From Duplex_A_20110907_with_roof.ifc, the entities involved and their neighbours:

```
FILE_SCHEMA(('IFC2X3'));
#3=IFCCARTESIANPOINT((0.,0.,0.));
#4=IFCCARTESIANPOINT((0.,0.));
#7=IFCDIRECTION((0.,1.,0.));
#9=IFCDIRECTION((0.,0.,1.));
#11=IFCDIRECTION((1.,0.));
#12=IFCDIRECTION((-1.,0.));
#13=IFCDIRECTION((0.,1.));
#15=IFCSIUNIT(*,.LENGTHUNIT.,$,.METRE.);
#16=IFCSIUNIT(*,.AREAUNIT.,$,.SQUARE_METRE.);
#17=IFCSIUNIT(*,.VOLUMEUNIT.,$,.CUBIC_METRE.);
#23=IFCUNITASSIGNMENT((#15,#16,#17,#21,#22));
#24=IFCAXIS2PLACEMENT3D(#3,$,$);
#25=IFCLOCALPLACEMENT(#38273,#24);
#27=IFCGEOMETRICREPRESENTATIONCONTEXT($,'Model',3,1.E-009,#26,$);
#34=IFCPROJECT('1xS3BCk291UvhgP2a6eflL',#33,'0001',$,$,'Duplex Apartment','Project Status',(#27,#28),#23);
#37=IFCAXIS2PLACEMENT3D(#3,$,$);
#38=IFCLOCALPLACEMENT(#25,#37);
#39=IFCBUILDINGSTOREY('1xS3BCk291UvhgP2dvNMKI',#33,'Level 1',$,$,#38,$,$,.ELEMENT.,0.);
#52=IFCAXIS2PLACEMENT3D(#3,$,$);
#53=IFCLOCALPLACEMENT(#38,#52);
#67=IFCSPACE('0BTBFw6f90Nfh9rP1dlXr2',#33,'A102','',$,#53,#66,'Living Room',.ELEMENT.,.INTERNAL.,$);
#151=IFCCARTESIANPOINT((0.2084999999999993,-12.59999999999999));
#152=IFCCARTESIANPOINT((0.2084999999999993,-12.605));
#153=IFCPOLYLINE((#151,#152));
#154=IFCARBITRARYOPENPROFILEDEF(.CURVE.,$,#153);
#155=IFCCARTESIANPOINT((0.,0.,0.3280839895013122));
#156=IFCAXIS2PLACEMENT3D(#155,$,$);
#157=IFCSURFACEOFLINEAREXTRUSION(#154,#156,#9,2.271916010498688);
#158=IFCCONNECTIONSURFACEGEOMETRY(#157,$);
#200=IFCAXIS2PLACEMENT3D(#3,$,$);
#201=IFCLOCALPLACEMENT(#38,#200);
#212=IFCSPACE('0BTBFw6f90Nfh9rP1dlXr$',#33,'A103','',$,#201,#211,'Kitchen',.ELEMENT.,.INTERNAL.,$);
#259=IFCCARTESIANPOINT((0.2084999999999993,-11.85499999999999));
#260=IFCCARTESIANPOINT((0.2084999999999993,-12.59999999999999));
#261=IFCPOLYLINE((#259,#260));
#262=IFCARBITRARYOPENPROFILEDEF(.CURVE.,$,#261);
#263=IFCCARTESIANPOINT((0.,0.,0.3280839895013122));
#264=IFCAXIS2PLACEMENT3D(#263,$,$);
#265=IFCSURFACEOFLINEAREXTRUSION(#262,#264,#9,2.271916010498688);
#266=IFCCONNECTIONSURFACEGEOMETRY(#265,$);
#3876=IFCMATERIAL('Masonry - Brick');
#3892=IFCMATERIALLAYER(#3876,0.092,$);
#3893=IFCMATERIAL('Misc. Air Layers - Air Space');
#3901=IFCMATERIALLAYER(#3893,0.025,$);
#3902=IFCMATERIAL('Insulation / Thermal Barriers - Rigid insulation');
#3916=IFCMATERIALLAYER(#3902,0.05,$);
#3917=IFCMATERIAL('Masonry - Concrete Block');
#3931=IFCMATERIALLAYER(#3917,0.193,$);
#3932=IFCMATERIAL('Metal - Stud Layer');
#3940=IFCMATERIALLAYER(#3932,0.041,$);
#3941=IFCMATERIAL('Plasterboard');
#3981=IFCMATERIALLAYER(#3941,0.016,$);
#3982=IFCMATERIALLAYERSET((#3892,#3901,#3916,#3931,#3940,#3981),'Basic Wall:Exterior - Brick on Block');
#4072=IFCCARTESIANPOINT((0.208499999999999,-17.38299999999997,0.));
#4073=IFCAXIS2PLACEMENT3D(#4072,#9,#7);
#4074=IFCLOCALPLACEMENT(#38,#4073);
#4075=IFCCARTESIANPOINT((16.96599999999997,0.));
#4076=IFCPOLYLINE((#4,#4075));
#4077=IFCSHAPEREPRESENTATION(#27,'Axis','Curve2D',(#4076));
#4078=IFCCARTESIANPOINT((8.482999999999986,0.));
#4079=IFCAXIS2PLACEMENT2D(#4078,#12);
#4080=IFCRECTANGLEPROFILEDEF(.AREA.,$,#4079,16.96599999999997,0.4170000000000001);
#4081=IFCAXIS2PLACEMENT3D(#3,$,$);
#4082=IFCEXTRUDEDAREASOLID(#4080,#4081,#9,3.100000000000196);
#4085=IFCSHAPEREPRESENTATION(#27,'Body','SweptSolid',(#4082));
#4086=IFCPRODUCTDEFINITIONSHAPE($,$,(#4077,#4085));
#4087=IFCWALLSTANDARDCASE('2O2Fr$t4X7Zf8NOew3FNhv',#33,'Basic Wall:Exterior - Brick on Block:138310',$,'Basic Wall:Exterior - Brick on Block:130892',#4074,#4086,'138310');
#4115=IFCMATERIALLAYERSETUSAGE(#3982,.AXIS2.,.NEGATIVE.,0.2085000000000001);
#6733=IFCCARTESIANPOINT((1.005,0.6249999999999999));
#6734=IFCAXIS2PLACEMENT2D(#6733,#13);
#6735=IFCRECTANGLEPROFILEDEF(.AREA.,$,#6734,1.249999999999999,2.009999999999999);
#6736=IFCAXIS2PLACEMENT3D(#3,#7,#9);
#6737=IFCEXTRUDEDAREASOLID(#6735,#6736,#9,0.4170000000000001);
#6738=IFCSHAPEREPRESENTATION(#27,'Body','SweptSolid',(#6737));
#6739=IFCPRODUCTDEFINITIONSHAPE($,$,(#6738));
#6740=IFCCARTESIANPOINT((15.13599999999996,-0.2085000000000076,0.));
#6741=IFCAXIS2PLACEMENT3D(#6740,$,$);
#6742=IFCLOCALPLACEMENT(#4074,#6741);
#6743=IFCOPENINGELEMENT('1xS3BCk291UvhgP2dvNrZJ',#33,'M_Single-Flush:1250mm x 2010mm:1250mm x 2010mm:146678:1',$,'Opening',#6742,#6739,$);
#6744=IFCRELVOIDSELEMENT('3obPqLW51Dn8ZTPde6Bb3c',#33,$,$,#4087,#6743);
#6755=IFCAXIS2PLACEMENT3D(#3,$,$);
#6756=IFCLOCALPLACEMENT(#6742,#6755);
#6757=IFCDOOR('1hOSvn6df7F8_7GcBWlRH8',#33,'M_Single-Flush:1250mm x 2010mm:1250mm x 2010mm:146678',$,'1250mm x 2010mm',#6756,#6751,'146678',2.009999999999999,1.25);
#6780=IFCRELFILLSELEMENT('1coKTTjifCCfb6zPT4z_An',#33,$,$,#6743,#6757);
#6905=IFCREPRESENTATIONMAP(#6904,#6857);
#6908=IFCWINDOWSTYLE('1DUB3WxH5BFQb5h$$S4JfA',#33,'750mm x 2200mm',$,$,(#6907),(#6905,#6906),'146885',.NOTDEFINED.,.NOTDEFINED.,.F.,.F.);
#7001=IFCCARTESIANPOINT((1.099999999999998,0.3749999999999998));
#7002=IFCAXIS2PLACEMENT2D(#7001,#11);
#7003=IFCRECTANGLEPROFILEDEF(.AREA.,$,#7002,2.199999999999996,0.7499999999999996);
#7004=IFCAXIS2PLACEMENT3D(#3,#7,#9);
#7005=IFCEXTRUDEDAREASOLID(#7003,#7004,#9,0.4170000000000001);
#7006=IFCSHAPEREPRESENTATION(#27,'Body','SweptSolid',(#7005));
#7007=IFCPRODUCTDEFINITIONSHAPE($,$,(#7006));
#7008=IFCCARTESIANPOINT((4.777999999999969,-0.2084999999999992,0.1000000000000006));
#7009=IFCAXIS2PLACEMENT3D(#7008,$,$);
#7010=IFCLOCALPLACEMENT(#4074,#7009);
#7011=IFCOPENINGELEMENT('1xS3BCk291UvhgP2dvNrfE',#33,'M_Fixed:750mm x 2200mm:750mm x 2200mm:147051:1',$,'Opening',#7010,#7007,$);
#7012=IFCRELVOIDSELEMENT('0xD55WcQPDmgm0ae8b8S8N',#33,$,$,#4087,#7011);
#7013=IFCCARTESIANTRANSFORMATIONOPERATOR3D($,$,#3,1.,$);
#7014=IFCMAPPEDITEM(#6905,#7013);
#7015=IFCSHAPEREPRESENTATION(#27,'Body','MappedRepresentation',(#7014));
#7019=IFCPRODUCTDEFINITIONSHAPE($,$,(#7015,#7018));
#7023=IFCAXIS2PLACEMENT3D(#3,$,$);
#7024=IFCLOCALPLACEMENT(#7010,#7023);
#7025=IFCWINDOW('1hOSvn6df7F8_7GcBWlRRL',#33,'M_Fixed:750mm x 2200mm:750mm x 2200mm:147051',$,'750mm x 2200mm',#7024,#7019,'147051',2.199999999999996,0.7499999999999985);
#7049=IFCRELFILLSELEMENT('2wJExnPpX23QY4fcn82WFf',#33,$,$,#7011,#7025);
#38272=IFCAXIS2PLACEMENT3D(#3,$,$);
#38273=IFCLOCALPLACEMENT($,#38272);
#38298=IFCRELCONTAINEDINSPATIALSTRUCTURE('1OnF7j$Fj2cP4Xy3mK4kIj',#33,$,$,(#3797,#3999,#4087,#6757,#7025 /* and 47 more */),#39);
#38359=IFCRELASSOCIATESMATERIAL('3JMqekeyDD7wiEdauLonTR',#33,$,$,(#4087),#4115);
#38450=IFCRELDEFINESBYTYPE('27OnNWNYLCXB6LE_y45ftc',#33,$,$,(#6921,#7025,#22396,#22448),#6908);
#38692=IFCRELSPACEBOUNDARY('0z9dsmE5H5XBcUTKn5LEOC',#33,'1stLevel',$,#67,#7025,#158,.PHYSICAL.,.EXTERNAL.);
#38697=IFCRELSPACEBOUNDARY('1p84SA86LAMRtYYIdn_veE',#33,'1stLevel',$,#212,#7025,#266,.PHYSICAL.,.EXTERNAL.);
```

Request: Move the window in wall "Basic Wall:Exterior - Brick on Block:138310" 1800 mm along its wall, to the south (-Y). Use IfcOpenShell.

```python
import numpy as np
import ifcopenshell
import ifcopenshell.api.geometry
import ifcopenshell.util.placement
import ifcopenshell.util.unit

model = ifcopenshell.open("Duplex_A_20110907_with_roof.ifc")
unit_scale = ifcopenshell.util.unit.calculate_unit_scale(model)

window = model.by_id(7025)
opening = window.FillsVoids[0].RelatingOpeningElement
wall = opening.VoidsElements[0].RelatingBuildingElement

wall_matrix = ifcopenshell.util.placement.get_local_placement(wall.ObjectPlacement)
shift = wall_matrix[:3, 0] * -1.8 / unit_scale
before = ifcopenshell.util.placement.get_local_placement(window.ObjectPlacement)[:3, 3].copy()

# The window is placed relative to its opening, so it follows when the opening moves.
matrix = ifcopenshell.util.placement.get_local_placement(opening.ObjectPlacement)
matrix[:3, 3] += shift
ifcopenshell.api.geometry.edit_object_placement(
    model, product=opening, matrix=matrix, is_si=False, should_transform_children=True
)

# Space boundary surfaces are stored in each space's coordinates; move them too.
for rel in window.ProvidesBoundaries:
    if not rel.ConnectionGeometry:
        continue
    surface = rel.ConnectionGeometry.SurfaceOnRelatingElement
    space_matrix = ifcopenshell.util.placement.get_local_placement(rel.RelatingSpace.ObjectPlacement)
    point = np.array(surface.Position.Location.Coordinates) + space_matrix[:3, :3].T @ shift
    surface.Position = model.createIfcAxis2Placement3D(
        model.createIfcCartesianPoint(point.tolist()), surface.Position.Axis, surface.Position.RefDirection
    )

after = ifcopenshell.util.placement.get_local_placement(window.ObjectPlacement)[:3, 3]
print("window moved by", (after - before).round(3) + 0.0)

model.write("Duplex_A_20110907_with_roof_rev.ifc")
```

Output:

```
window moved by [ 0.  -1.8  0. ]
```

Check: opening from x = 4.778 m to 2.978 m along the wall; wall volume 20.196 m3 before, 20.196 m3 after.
